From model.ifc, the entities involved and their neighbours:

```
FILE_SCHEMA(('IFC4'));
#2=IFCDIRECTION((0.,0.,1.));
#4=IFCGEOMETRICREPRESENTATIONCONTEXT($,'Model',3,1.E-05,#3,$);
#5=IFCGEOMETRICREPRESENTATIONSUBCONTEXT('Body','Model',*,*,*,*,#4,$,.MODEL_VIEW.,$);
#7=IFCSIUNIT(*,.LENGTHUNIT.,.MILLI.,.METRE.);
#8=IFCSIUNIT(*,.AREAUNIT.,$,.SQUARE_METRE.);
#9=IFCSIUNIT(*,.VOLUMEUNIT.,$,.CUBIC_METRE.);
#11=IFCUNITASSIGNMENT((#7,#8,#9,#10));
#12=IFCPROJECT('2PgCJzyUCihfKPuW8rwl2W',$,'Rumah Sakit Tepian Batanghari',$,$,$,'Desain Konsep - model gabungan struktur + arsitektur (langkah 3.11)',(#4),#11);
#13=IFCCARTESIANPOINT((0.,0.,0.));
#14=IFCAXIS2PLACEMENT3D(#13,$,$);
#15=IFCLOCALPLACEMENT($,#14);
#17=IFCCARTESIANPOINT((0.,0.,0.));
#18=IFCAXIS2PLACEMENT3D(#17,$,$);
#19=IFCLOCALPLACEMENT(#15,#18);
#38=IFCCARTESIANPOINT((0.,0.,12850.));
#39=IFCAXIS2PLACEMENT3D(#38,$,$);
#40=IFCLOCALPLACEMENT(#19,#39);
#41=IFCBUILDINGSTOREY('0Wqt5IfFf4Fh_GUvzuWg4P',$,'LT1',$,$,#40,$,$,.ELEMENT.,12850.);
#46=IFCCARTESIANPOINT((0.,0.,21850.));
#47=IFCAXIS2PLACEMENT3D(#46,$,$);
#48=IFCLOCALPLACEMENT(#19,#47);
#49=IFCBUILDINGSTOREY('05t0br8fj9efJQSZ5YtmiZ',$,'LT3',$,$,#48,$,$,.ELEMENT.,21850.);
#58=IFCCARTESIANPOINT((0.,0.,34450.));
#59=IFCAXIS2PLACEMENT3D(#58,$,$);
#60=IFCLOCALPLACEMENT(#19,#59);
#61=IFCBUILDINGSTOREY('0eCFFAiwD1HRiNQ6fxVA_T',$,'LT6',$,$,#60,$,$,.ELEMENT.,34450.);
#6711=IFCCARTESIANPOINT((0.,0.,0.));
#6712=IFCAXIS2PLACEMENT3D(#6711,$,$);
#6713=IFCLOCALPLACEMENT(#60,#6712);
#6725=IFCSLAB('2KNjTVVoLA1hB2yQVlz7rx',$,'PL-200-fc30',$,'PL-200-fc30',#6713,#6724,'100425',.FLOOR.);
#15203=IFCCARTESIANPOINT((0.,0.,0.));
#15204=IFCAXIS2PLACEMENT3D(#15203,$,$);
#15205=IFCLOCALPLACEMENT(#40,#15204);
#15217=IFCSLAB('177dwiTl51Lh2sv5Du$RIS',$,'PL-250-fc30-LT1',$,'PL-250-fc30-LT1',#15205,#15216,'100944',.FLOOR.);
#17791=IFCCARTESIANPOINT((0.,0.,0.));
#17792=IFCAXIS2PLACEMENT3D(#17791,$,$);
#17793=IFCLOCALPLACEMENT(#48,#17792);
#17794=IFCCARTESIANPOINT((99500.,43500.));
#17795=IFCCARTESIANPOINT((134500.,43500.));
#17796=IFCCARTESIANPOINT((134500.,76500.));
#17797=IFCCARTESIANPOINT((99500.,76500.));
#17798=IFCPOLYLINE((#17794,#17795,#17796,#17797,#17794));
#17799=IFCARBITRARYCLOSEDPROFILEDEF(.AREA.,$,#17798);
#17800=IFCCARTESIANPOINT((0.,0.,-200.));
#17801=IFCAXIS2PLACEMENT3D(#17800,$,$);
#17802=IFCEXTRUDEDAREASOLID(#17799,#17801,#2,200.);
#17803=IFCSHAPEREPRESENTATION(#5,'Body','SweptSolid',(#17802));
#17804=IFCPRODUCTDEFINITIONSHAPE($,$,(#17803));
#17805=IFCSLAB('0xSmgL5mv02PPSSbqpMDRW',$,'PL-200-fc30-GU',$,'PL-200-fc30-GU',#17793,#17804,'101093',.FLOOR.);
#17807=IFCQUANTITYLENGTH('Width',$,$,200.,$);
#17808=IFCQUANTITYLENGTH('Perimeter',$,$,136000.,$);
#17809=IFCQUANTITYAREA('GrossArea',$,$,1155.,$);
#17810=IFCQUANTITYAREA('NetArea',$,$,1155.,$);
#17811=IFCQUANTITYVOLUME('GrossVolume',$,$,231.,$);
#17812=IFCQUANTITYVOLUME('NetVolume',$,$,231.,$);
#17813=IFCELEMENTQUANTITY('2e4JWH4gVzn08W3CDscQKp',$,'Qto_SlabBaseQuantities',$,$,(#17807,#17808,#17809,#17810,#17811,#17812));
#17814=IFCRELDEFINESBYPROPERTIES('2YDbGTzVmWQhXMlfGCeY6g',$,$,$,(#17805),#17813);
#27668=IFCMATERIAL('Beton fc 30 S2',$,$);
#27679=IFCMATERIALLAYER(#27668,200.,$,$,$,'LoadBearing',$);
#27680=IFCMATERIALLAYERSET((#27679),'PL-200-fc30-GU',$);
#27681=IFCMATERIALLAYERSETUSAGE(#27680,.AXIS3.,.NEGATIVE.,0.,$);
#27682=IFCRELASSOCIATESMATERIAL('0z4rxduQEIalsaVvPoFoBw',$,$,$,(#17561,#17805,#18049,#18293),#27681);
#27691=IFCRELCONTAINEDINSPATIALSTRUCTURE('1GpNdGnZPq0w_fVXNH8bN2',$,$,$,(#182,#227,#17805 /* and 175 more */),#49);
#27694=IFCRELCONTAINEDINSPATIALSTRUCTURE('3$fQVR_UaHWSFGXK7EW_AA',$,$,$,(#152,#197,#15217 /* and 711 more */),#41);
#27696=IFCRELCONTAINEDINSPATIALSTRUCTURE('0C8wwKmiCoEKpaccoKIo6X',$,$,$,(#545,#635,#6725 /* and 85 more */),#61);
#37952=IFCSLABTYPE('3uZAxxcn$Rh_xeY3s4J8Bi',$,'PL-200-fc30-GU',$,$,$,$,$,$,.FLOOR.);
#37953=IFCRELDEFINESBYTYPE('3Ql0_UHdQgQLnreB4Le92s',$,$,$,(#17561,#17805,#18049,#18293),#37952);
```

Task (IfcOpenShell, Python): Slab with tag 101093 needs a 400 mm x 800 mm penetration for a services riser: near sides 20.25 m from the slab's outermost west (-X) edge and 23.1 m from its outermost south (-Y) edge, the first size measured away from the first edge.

```python
import numpy as np
import ifcopenshell
import ifcopenshell.api.feature
import ifcopenshell.api.geometry
import ifcopenshell.api.pset
import ifcopenshell.api.root
import ifcopenshell.geom
import ifcopenshell.util.element
import ifcopenshell.util.placement
import ifcopenshell.util.representation
import ifcopenshell.util.shape
import ifcopenshell.util.unit

model = ifcopenshell.open("model.ifc")
unit_scale = ifcopenshell.util.unit.calculate_unit_scale(model)
area_scale = ifcopenshell.util.unit.calculate_unit_scale(model, "AREAUNIT")
volume_scale = ifcopenshell.util.unit.calculate_unit_scale(model, "VOLUMEUNIT")
settings = ifcopenshell.geom.settings()


def volume(element):
    """Net volume in cubic metres, openings subtracted."""
    shape = ifcopenshell.geom.create_shape(settings, element)
    return ifcopenshell.util.shape.get_volume(shape.geometry)


slab = model.by_guid("0xSmgL5mv02PPSSbqpMDRW")
before = volume(slab)

# Extent in the slab's own axes, in metres. The edges named are its -X and -Y sides.
slab_shape = ifcopenshell.geom.create_shape(settings, slab)
vertices = ifcopenshell.util.shape.get_vertices(slab_shape.geometry)
x_min, y_min, bottom = vertices.min(axis=0)
top = vertices[:, 2].max()

opening = ifcopenshell.api.root.create_entity(model, ifc_class="IfcOpeningElement", name="Services riser opening", predefined_type="OPENING")
context = ifcopenshell.util.representation.get_context(model, "Model", "Body", "MODEL_VIEW")
width, depth = 0.4, 0.8
outline = [(0.0, 0.0), (width, 0.0), (width, depth), (0.0, depth), (0.0, 0.0)]
# Overshoot both faces by 50 mm so the cut is clean.
shape = ifcopenshell.api.geometry.add_slab_representation(
    model, context=context, depth=top - bottom + 0.1, polyline=outline
)
ifcopenshell.api.geometry.assign_representation(model, product=opening, representation=shape)

matrix = ifcopenshell.util.placement.get_local_placement(slab.ObjectPlacement)
matrix[:, 3] = matrix @ np.append(np.array([x_min + 20.25, y_min + 23.1, bottom - 0.05]) / unit_scale, 1.0)
ifcopenshell.api.geometry.edit_object_placement(model, product=opening, matrix=matrix, is_si=False)
ifcopenshell.api.feature.add_feature(model, feature=opening, element=slab)

after = volume(slab)

# Update the slab's stored quantities.
qto = model.by_id(ifcopenshell.util.element.get_pset(slab, "Qto_SlabBaseQuantities", should_inherit=False)["id"])
ifcopenshell.api.pset.edit_qto(model, qto=qto, properties={
    "NetArea": after / (top - bottom) / area_scale,
    "NetVolume": after / volume_scale,
})

print(f"slab volume {before:.3f} -> {after:.3f} m3")

model.write("model_rev.ifc")
```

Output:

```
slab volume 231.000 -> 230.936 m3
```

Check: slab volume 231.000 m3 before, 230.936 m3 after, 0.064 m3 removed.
